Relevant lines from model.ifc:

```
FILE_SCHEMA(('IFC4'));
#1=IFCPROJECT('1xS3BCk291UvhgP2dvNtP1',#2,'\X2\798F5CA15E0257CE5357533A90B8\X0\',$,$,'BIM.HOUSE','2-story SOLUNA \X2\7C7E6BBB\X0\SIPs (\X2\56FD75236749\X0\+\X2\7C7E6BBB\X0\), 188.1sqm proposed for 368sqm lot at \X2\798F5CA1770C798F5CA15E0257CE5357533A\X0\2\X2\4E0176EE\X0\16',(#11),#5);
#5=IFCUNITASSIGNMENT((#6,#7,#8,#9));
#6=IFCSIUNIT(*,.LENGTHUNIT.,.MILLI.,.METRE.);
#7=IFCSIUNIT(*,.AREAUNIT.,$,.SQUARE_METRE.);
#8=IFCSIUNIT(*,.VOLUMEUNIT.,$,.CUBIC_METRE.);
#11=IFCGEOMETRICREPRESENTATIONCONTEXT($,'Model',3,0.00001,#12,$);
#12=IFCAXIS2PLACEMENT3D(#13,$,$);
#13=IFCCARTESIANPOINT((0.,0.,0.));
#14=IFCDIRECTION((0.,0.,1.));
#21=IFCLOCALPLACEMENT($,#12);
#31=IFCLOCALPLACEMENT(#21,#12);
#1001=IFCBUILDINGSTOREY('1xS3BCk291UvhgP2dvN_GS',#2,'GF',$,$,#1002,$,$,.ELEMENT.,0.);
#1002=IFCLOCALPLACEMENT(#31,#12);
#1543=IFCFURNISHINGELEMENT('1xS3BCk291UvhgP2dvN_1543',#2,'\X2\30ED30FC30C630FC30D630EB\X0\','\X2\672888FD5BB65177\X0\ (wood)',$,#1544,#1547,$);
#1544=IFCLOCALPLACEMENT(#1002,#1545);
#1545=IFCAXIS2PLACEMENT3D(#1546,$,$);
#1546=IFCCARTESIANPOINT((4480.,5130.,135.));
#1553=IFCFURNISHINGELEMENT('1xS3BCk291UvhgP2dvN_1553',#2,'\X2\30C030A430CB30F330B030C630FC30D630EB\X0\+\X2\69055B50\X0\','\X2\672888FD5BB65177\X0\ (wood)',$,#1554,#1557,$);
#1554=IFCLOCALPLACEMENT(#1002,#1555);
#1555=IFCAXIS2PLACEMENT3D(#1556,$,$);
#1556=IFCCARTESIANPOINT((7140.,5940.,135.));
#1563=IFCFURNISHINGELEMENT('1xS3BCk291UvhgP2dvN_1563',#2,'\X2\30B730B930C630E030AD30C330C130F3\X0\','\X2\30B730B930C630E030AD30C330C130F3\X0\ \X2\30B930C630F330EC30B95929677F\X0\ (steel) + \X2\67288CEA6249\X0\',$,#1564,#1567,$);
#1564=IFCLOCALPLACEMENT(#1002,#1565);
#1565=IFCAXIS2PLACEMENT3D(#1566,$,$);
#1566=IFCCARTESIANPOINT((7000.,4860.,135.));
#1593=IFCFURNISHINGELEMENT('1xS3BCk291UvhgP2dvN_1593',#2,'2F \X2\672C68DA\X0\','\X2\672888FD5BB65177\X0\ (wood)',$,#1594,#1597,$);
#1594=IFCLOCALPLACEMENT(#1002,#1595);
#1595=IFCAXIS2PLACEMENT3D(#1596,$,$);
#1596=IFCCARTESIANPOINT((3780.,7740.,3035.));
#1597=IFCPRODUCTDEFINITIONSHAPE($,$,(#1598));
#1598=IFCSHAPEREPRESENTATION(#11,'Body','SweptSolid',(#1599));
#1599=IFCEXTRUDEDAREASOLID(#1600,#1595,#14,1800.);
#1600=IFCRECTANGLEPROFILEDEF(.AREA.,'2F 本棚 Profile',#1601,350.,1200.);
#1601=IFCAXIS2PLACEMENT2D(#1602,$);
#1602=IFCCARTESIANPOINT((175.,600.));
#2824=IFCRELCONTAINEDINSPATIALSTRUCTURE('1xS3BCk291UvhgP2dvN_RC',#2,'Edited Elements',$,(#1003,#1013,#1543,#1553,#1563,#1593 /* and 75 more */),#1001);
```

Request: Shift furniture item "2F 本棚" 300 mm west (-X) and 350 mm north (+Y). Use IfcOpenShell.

```python
import ifcopenshell
import ifcopenshell.api.geometry
import ifcopenshell.util.placement
import ifcopenshell.util.unit

model = ifcopenshell.open("model.ifc")
unit_scale = ifcopenshell.util.unit.calculate_unit_scale(model)

item = model.by_id(1593)
matrix = ifcopenshell.util.placement.get_local_placement(item.ObjectPlacement)
matrix[0, 3] -= 0.3 / unit_scale
matrix[1, 3] += 0.35 / unit_scale
ifcopenshell.api.geometry.edit_object_placement(model, product=item, matrix=matrix, is_si=False)

print(ifcopenshell.util.placement.get_local_placement(item.ObjectPlacement).round(3) + 0.0)

model.write("model_edited.ifc")
```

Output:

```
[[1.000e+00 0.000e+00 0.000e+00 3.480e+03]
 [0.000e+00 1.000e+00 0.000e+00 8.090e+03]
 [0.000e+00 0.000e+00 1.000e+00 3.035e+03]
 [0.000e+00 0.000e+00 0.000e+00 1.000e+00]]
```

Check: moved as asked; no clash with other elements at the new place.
